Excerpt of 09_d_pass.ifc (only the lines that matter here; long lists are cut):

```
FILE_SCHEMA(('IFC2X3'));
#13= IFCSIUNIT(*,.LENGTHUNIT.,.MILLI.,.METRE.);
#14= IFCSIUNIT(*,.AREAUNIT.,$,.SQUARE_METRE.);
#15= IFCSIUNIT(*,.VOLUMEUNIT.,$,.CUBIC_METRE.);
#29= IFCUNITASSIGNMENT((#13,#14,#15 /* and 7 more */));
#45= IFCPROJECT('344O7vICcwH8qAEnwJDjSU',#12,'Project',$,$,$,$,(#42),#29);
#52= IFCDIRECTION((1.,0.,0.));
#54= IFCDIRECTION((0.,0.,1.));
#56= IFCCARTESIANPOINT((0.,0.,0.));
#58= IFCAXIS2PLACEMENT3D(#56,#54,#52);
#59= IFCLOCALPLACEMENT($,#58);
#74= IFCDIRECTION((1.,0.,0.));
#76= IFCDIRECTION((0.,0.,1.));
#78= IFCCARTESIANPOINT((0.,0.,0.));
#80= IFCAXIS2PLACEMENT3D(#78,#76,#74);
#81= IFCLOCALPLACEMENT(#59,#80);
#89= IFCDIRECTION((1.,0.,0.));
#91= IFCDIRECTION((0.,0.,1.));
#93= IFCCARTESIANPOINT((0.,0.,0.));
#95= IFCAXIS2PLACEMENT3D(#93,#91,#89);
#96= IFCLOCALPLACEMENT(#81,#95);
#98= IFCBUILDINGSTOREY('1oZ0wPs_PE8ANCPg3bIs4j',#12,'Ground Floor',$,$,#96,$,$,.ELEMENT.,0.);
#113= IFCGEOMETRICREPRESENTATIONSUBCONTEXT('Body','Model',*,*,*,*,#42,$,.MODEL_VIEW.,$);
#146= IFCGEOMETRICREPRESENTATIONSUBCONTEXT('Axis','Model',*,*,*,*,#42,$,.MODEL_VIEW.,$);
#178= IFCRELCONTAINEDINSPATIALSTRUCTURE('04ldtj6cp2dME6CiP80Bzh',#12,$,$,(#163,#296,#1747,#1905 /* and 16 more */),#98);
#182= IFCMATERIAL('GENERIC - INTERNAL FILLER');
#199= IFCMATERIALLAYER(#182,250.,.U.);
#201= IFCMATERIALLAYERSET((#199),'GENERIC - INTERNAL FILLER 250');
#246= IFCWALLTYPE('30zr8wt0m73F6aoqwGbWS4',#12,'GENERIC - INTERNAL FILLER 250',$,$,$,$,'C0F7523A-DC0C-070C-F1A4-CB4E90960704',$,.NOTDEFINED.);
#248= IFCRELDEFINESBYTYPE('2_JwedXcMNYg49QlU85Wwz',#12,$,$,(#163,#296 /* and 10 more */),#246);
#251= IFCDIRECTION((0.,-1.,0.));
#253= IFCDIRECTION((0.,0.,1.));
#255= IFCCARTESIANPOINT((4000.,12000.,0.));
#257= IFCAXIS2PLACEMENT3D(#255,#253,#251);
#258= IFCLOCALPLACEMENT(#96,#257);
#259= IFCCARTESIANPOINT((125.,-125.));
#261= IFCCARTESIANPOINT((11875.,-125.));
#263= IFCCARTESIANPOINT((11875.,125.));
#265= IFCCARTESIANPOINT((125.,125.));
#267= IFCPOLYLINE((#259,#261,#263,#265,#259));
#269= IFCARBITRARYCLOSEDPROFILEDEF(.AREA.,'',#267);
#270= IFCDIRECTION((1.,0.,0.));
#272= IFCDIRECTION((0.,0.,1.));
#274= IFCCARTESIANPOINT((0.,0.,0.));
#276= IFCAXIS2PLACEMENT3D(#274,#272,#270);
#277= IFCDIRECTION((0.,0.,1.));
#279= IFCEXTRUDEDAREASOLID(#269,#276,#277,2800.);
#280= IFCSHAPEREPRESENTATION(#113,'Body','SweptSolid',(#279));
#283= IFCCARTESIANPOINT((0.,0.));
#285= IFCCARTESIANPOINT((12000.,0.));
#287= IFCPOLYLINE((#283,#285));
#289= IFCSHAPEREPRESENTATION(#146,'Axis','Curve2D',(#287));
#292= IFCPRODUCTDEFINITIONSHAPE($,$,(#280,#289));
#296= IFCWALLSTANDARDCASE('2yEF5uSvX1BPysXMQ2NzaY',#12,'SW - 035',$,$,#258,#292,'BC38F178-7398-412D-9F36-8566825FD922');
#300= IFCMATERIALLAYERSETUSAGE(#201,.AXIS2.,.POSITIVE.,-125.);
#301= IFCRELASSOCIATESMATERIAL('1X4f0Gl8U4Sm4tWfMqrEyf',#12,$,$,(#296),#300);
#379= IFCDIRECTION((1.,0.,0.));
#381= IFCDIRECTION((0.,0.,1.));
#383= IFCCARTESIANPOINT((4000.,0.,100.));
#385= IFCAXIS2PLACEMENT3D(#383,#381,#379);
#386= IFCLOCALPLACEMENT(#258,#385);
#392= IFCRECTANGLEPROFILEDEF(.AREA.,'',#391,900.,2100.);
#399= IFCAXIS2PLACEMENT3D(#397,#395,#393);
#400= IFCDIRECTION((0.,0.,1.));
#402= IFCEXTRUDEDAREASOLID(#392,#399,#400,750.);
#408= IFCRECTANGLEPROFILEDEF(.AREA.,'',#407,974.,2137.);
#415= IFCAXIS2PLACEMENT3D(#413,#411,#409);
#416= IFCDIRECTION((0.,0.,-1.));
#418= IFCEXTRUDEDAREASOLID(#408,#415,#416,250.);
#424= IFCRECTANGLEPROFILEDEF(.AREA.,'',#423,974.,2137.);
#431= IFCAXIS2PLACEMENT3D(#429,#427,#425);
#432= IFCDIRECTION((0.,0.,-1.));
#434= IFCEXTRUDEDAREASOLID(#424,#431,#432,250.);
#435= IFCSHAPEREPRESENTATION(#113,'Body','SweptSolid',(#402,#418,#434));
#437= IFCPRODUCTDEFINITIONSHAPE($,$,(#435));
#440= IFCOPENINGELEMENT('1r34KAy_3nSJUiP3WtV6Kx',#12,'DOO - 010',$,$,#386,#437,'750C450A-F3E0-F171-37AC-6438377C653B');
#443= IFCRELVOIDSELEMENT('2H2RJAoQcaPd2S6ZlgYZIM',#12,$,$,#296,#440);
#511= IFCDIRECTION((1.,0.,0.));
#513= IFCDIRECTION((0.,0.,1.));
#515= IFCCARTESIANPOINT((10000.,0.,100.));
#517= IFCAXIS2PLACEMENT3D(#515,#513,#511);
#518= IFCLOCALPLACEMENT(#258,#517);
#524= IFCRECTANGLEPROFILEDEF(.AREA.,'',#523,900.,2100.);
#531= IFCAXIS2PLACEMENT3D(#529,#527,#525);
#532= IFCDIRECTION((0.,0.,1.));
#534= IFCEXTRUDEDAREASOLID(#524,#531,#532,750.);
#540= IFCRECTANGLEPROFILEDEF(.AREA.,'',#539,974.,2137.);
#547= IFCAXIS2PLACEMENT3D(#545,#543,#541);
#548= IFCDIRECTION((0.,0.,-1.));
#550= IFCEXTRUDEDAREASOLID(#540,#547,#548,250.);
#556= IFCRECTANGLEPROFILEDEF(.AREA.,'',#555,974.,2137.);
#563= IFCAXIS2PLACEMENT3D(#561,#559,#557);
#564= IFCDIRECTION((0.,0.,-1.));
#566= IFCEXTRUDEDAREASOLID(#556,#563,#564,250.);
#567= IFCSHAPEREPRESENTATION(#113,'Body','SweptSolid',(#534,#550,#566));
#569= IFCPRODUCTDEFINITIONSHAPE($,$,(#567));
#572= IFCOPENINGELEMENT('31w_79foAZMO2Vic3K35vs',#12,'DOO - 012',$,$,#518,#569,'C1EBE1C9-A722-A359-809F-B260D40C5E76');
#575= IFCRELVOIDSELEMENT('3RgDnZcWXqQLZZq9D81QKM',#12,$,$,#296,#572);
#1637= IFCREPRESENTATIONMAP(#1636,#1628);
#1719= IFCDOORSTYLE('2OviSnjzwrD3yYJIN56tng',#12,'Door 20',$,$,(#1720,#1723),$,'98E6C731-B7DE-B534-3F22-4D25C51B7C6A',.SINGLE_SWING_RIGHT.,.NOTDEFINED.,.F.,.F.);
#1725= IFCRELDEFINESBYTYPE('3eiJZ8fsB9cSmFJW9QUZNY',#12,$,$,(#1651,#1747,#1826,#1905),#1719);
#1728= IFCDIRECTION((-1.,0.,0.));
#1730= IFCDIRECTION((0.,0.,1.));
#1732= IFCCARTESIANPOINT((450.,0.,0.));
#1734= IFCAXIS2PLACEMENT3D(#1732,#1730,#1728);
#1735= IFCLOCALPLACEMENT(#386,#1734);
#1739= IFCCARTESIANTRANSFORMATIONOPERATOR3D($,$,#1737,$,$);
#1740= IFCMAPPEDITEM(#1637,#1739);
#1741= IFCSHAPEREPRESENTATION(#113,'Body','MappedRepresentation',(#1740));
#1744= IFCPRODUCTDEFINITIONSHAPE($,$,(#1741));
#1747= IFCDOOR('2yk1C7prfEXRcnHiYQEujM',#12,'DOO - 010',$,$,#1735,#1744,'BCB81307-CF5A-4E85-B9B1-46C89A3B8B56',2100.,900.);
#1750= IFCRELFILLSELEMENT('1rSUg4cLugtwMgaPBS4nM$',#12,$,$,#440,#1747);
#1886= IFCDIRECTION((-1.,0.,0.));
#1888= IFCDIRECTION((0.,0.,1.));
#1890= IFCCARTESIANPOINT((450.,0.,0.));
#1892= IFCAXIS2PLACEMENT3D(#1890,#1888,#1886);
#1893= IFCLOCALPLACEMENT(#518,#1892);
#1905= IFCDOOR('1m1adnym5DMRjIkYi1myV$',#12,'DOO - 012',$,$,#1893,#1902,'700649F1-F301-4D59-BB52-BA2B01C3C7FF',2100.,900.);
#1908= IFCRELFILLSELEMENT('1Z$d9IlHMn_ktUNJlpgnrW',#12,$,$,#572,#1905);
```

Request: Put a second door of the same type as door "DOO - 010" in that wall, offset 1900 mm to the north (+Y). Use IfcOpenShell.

```python
import ifcopenshell
import ifcopenshell.api.feature
import ifcopenshell.api.geometry
import ifcopenshell.api.root
import ifcopenshell.geom
import ifcopenshell.util.element
import ifcopenshell.util.placement
import ifcopenshell.util.shape

model = ifcopenshell.open("09_d_pass.ifc")
settings = ifcopenshell.geom.settings()


def volume(element):
    """Net volume in cubic metres, openings subtracted."""
    shape = ifcopenshell.geom.create_shape(settings, element)
    return ifcopenshell.util.shape.get_volume(shape.geometry)


def reuse_history(source, copy):
    """copy_class also copies each property set's owner history, people and application; keep the originals."""
    for rel in copy.IsDefinedBy:
        if rel.is_a("IfcRelDefinesByProperties") and (history := rel.RelatingPropertyDefinition.OwnerHistory):
            rel.RelatingPropertyDefinition.OwnerHistory = source.OwnerHistory
            ifcopenshell.util.element.remove_deep2(model, history)


door = model.by_guid("2yk1C7prfEXRcnHiYQEujM")
opening = door.FillsVoids[0].RelatingOpeningElement
wall = opening.VoidsElements[0].RelatingBuildingElement
before = volume(wall)
shift = ifcopenshell.util.placement.get_local_placement(wall.ObjectPlacement)[:3, 0] * -1900.0

# copy_class copies the void relationship, type, container and properties, but no geometry.
new_opening = ifcopenshell.api.root.copy_class(model, product=opening)
new_opening.Representation = ifcopenshell.util.element.copy_deep(
    model, opening.Representation, exclude=["IfcGeometricRepresentationContext", "IfcRepresentationMap"]
)
new_opening.Tag = None
new_door = ifcopenshell.api.root.copy_class(model, product=door)
new_door.Representation = ifcopenshell.util.element.copy_deep(
    model, door.Representation, exclude=["IfcGeometricRepresentationContext", "IfcRepresentationMap"]
)
new_door.Tag = None
reuse_history(door, new_door)
fills = ifcopenshell.api.feature.add_filling(model, opening=new_opening, element=new_door)
fills.OwnerHistory = new_door.OwnerHistory  # required in IFC2X3

for old, new in ((opening, new_opening), (door, new_door)):
    matrix = ifcopenshell.util.placement.get_local_placement(old.ObjectPlacement)
    matrix[:3, 3] += shift
    ifcopenshell.api.geometry.edit_object_placement(model, product=new, matrix=matrix, is_si=False)

after = volume(wall)

print(f"wall volume {before:.3f} -> {after:.3f} m3")

model.write("09_d_pass_edited.ifc")
```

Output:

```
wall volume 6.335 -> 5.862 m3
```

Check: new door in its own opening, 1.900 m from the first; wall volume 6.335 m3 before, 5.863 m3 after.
